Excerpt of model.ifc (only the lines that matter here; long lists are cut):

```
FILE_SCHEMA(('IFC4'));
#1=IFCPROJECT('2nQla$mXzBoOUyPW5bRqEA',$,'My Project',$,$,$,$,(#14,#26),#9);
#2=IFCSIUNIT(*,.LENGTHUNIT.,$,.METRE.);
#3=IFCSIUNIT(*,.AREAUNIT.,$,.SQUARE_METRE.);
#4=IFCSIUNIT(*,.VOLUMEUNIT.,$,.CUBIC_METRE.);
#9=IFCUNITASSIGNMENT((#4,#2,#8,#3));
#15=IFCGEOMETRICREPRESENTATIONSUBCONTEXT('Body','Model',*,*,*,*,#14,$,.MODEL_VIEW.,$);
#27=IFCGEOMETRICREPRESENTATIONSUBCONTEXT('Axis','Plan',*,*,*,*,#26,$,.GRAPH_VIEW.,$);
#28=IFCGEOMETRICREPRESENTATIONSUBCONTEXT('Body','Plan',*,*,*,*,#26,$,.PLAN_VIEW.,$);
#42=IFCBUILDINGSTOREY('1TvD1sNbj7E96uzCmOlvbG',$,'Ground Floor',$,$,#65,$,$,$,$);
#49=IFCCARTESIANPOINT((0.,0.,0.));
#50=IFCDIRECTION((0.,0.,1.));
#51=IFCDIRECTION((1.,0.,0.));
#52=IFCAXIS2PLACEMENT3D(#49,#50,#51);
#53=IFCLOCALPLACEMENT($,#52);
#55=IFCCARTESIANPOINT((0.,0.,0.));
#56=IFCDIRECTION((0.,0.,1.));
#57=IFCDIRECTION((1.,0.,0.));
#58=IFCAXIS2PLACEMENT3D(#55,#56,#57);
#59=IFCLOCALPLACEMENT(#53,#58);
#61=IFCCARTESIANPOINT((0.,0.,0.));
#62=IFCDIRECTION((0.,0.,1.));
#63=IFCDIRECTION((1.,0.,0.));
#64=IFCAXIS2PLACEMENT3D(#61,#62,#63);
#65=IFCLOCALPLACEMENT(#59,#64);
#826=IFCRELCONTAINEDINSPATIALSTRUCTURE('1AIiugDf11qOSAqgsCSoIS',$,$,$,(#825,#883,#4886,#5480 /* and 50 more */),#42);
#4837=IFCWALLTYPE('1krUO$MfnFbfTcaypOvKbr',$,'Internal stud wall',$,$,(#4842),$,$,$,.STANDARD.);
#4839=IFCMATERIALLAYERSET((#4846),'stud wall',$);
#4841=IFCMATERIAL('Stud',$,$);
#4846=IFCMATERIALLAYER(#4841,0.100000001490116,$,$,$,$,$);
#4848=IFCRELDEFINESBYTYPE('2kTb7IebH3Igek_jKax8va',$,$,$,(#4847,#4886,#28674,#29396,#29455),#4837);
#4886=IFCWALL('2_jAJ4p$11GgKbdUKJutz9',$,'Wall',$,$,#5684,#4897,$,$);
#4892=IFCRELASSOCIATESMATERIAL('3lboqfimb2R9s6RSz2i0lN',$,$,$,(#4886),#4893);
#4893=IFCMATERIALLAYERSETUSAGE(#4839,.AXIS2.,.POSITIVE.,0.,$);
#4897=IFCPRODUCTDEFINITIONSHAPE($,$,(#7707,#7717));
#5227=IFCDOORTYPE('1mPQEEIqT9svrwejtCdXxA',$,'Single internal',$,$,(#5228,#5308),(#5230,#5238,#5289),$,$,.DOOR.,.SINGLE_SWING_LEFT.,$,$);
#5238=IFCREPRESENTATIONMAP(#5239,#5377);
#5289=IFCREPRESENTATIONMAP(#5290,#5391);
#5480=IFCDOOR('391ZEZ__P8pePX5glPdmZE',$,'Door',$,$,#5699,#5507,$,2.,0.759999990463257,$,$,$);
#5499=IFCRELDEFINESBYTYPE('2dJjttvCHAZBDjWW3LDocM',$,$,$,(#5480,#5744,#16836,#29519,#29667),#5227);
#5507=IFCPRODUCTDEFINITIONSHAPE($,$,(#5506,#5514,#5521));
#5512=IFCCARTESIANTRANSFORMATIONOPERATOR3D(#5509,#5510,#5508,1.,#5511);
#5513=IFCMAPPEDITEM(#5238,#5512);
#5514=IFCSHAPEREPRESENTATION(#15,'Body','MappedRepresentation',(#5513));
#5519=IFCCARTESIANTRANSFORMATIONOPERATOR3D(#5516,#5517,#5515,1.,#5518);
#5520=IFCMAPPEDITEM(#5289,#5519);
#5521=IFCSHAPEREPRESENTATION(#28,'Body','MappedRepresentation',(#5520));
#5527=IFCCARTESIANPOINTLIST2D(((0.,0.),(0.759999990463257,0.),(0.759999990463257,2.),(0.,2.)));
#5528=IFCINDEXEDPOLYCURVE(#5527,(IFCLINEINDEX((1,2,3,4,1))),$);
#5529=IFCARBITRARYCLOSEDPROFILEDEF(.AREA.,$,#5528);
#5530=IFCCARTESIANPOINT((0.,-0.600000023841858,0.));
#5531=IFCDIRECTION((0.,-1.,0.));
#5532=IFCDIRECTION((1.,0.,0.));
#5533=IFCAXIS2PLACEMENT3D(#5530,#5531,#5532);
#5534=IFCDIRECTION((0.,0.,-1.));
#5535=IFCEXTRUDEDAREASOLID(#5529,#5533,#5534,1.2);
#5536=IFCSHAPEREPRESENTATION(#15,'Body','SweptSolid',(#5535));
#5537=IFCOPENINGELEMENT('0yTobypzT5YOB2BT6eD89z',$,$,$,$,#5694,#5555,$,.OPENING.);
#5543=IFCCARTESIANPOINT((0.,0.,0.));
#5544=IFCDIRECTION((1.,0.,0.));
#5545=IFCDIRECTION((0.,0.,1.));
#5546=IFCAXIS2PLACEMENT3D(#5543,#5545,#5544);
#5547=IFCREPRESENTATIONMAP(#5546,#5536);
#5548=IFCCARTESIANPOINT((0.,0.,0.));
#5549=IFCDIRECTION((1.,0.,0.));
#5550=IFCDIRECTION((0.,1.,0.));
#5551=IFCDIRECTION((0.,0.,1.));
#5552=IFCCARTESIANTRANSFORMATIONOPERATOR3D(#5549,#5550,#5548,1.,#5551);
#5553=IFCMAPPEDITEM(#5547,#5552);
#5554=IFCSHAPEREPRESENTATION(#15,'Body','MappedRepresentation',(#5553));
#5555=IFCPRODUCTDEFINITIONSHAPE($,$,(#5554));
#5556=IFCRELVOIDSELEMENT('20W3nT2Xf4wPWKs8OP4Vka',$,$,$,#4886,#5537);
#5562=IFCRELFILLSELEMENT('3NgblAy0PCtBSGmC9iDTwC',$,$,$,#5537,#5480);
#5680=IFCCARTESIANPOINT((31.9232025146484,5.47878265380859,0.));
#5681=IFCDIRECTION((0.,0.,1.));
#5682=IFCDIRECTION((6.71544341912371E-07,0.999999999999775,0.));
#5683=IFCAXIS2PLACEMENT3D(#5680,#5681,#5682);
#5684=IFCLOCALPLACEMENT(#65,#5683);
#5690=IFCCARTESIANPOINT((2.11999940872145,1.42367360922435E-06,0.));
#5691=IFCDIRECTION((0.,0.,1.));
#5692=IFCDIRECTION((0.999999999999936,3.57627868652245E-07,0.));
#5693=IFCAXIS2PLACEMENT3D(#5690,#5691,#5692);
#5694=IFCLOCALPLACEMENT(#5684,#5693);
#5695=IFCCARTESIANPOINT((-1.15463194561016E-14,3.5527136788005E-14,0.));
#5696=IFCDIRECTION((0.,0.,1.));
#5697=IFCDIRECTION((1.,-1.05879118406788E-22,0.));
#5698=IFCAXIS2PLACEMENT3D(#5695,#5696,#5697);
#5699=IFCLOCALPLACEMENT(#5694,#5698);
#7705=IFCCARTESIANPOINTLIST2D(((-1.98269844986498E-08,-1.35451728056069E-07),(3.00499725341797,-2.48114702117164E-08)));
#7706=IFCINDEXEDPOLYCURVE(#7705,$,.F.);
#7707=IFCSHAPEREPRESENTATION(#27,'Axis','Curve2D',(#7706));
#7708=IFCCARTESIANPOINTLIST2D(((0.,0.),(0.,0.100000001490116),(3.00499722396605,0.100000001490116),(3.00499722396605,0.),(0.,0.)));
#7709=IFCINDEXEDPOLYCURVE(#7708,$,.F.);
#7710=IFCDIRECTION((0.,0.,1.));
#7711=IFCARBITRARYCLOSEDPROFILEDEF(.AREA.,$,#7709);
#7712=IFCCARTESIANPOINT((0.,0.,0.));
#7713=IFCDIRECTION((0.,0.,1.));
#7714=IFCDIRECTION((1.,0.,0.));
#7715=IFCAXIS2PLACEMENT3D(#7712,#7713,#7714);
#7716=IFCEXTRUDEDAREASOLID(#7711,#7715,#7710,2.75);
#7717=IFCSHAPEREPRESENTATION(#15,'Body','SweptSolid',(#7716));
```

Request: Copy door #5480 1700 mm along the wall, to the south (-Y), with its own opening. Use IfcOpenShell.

```python
import ifcopenshell
import ifcopenshell.api.feature
import ifcopenshell.api.geometry
import ifcopenshell.api.root
import ifcopenshell.geom
import ifcopenshell.util.element
import ifcopenshell.util.placement
import ifcopenshell.util.shape
import ifcopenshell.util.unit

model = ifcopenshell.open("model.ifc")
unit_scale = ifcopenshell.util.unit.calculate_unit_scale(model)
settings = ifcopenshell.geom.settings()


def volume(element):
    """Net volume in cubic metres, openings subtracted."""
    shape = ifcopenshell.geom.create_shape(settings, element)
    return ifcopenshell.util.shape.get_volume(shape.geometry)


door = model.by_guid("391ZEZ__P8pePX5glPdmZE")
opening = door.FillsVoids[0].RelatingOpeningElement
wall = opening.VoidsElements[0].RelatingBuildingElement
before = volume(wall)
shift = ifcopenshell.util.placement.get_local_placement(wall.ObjectPlacement)[:3, 0] * -1.7 / unit_scale

# copy_class copies the void relationship, type, container and properties, but no geometry.
new_opening = ifcopenshell.api.root.copy_class(model, product=opening)
new_opening.Representation = ifcopenshell.util.element.copy_deep(
    model, opening.Representation, exclude=["IfcGeometricRepresentationContext", "IfcRepresentationMap"]
)
new_door = ifcopenshell.api.root.copy_class(model, product=door)
new_door.Representation = ifcopenshell.util.element.copy_deep(
    model, door.Representation, exclude=["IfcGeometricRepresentationContext", "IfcRepresentationMap"]
)
ifcopenshell.api.feature.add_filling(model, opening=new_opening, element=new_door)

for old, new in ((opening, new_opening), (door, new_door)):
    matrix = ifcopenshell.util.placement.get_local_placement(old.ObjectPlacement)
    matrix[:3, 3] += shift
    ifcopenshell.api.geometry.edit_object_placement(model, product=new, matrix=matrix, is_si=False)

after = volume(wall)

print(f"wall volume {before:.3f} -> {after:.3f} m3")

model.write("model-out.ifc")
```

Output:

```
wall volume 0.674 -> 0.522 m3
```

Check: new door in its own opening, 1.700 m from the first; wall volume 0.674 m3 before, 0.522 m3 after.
